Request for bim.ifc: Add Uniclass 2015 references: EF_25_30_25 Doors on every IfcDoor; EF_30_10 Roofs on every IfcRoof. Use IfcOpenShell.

First a look at what the model holds.

```python
import ifcopenshell

model = ifcopenshell.open("bim.ifc")
print(model.schema)
print("classifications:", [c.Name for c in model.by_type("IfcClassification")])
for ifc_class in ("IfcDoor", "IfcRoof", "IfcStair", "IfcWall", "IfcWindow"):
    print(ifc_class, len(model.by_type(ifc_class)))
```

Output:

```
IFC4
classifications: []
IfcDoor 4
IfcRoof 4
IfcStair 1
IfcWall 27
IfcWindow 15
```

```python
import ifcopenshell
import ifcopenshell.api.classification

model = ifcopenshell.open("bim.ifc")

system = ifcopenshell.api.classification.add_classification(model, classification="Uniclass 2015")

codes = {
    "IfcDoor": ("EF_25_30_25", "Doors"),
    "IfcRoof": ("EF_30_10", "Roofs"),
}
for ifc_class, (code, name) in codes.items():
    products = model.by_type(ifc_class)
    ifcopenshell.api.classification.add_reference(
        model, products=products, classification=system, identification=code, name=name
    )
    print(code, len(products))

model.write("bim-out.ifc")
```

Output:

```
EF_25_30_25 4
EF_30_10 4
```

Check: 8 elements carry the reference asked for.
